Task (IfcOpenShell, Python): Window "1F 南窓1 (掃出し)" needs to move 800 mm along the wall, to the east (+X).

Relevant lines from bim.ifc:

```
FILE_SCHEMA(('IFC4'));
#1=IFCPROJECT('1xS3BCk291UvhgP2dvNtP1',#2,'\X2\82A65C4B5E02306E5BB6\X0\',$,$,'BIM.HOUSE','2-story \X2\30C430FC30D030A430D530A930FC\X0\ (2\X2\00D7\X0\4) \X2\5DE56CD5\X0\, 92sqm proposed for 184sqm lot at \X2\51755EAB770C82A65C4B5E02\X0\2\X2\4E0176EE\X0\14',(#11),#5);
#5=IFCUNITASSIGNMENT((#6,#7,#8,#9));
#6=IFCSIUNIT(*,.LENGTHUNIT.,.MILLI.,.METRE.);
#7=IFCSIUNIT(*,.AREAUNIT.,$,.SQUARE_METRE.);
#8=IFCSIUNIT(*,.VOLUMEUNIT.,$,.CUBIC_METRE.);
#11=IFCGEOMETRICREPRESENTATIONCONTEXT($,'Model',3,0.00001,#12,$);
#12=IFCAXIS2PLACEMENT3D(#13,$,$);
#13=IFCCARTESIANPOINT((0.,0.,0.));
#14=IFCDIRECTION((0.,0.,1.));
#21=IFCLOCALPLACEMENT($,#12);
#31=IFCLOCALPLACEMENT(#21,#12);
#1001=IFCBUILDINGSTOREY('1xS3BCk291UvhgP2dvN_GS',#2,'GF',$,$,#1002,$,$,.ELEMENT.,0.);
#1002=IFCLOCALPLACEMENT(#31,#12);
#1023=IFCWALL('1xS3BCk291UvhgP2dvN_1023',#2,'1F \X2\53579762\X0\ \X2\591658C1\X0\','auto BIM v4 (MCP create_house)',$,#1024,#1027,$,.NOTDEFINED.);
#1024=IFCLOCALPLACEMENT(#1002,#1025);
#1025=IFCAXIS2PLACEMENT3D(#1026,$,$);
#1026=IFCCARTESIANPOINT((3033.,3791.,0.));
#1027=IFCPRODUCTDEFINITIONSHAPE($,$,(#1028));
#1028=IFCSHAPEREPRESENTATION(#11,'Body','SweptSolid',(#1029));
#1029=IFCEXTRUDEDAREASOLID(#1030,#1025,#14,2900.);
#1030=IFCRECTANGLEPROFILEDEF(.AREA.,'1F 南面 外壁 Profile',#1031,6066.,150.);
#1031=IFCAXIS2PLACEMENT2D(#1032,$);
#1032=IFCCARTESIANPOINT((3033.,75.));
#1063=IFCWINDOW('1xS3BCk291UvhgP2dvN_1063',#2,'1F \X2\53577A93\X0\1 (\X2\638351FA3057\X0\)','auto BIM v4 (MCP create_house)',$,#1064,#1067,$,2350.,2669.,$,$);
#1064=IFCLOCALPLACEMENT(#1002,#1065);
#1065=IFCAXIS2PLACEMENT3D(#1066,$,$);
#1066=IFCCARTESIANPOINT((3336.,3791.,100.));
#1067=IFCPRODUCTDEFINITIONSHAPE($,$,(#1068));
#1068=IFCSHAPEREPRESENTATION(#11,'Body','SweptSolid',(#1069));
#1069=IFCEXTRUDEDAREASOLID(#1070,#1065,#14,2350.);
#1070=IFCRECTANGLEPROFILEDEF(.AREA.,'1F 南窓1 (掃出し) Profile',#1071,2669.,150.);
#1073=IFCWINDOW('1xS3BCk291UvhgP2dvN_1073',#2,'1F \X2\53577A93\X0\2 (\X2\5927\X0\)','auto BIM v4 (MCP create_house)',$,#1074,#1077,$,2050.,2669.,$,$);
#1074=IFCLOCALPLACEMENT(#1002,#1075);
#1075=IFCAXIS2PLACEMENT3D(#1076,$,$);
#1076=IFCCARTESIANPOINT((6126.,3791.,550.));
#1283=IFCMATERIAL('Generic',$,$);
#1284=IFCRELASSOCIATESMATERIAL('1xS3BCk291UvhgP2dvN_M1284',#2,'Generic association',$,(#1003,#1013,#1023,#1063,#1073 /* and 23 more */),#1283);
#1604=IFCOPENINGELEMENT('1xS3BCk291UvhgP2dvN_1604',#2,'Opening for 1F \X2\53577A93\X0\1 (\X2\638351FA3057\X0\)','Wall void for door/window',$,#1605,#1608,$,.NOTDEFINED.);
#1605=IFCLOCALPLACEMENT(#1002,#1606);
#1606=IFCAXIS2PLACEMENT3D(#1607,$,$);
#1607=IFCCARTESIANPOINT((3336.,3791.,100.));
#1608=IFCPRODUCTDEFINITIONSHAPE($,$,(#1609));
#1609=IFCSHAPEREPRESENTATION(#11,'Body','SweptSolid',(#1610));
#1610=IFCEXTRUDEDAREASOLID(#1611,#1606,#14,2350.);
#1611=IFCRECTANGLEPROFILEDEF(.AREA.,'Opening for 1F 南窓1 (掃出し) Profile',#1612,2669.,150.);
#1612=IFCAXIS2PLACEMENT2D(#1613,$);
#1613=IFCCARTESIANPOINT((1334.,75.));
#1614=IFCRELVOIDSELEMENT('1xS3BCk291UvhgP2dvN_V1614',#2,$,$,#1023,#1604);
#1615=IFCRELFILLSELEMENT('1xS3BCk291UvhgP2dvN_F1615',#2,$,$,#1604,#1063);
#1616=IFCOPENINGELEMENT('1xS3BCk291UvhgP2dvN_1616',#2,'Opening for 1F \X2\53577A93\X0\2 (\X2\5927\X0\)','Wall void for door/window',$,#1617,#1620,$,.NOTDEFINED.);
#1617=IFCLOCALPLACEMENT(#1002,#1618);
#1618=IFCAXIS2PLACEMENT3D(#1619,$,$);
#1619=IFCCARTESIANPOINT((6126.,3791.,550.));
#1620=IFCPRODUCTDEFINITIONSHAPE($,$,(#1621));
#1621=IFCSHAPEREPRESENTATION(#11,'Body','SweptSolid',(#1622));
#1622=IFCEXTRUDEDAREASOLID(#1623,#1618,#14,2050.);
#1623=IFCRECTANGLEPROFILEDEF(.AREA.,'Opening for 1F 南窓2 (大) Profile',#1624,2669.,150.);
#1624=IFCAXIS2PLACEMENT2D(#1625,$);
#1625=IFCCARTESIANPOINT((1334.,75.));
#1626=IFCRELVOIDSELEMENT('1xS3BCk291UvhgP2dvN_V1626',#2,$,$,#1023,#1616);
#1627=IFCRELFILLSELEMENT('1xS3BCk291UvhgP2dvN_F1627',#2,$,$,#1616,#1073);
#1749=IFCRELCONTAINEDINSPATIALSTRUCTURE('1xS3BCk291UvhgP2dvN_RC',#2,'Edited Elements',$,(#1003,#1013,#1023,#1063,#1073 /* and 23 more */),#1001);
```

```python
import ifcopenshell
import ifcopenshell.api.geometry
import ifcopenshell.util.placement

model = ifcopenshell.open("bim.ifc")

window = model.by_id(1063)
opening = window.FillsVoids[0].RelatingOpeningElement
wall = opening.VoidsElements[0].RelatingBuildingElement

wall_matrix = ifcopenshell.util.placement.get_local_placement(wall.ObjectPlacement)
shift = wall_matrix[:3, 0] * 800.0
before = ifcopenshell.util.placement.get_local_placement(window.ObjectPlacement)[:3, 3].copy()

# The window is not placed relative to its opening, so move both.
for product in (opening, window):
    matrix = ifcopenshell.util.placement.get_local_placement(product.ObjectPlacement)
    matrix[:3, 3] += shift
    ifcopenshell.api.geometry.edit_object_placement(model, product=product, matrix=matrix, is_si=False)

after = ifcopenshell.util.placement.get_local_placement(window.ObjectPlacement)[:3, 3]
print("window moved by", (after - before).round(3) + 0.0)

model.write("bim_updated.ifc")
```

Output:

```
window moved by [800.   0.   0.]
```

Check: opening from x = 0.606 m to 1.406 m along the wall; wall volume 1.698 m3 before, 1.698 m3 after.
